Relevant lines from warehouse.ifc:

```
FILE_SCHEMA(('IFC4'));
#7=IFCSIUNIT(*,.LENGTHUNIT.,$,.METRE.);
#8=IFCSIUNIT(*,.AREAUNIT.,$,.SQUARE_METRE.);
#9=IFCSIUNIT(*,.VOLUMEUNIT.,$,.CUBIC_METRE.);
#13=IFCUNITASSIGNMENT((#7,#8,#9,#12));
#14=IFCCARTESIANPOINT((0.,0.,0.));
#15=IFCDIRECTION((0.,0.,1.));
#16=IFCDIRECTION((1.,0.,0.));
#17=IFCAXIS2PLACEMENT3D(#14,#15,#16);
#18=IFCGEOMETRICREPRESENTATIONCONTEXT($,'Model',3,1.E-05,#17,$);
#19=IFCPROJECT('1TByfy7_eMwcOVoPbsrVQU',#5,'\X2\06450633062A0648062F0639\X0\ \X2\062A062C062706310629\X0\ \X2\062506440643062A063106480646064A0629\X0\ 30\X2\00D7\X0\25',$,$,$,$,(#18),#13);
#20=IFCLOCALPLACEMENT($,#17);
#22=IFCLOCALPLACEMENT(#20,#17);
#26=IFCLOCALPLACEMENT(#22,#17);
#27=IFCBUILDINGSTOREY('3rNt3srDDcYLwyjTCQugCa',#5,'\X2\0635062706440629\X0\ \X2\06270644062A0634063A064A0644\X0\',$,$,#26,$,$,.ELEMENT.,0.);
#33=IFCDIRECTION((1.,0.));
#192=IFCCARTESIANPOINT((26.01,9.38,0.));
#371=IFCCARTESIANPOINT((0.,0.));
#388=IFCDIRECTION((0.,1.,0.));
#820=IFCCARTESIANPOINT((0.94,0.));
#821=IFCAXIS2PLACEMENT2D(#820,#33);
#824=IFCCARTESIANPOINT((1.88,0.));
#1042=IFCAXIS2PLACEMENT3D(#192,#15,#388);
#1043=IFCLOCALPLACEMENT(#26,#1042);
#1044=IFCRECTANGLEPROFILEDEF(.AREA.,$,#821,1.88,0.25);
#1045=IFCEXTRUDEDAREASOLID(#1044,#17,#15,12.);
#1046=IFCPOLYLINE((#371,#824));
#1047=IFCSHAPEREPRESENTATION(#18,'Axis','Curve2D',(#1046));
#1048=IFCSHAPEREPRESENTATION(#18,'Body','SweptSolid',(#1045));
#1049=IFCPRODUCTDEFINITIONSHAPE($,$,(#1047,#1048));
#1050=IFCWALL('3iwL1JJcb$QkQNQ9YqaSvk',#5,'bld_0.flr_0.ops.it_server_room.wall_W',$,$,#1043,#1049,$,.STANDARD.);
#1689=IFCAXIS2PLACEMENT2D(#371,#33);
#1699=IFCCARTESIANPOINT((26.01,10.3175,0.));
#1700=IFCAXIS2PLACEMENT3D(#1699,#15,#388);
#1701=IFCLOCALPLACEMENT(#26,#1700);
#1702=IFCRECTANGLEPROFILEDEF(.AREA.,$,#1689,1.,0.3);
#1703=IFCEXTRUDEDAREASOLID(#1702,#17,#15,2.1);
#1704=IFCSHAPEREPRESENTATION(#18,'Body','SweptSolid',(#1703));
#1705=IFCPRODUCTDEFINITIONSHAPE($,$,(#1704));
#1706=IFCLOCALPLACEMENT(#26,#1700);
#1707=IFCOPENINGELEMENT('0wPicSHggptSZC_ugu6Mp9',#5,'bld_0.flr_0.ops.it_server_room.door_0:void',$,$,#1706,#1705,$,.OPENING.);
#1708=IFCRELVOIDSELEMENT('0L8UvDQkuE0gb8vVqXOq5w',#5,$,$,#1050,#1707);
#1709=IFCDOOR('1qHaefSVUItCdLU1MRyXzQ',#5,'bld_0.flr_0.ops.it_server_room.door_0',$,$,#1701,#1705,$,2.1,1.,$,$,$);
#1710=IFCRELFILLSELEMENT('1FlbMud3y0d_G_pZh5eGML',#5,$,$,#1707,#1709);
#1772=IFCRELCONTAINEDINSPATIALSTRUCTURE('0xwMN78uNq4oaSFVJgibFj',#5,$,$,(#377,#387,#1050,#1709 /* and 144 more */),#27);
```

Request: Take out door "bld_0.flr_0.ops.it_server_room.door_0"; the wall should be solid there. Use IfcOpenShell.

```python
import ifcopenshell
import ifcopenshell.api.feature
import ifcopenshell.api.root
import ifcopenshell.geom
import ifcopenshell.util.shape

model = ifcopenshell.open("warehouse.ifc")
settings = ifcopenshell.geom.settings()


def volume(element):
    """Net volume in cubic metres, openings subtracted."""
    shape = ifcopenshell.geom.create_shape(settings, element)
    return ifcopenshell.util.shape.get_volume(shape.geometry)


door = model.by_guid("1qHaefSVUItCdLU1MRyXzQ")
opening = door.FillsVoids[0].RelatingOpeningElement
wall = opening.VoidsElements[0].RelatingBuildingElement
before = volume(wall)

ifcopenshell.api.root.remove_product(model, product=door)
ifcopenshell.api.feature.remove_feature(model, feature=opening)

after = volume(wall)

print(f"wall volume {before:.3f} -> {after:.3f} m3")

model.write("warehouse_v2.ifc")
```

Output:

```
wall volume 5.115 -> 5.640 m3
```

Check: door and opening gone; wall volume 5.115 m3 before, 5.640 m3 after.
